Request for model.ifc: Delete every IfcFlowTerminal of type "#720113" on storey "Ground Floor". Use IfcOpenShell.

First a look at what the model holds.

```python
import ifcopenshell
import ifcopenshell.util.element

model = ifcopenshell.open("model.ifc")
print(model.schema)
storey = next(s for s in model.by_type("IfcBuildingStorey") if s.Name == "Ground Floor")
terminals = [e for e in ifcopenshell.util.element.get_decomposition(storey) if e.is_a("IfcFlowTerminal")]
seen = {}
for e in terminals:
    element_type = ifcopenshell.util.element.get_type(e)
    name = element_type.Name if element_type not in (None, e) else None
    seen[name] = seen.get(name, 0) + 1
for name, count in sorted(seen.items(), key=str):
    print(count, "x", name)
```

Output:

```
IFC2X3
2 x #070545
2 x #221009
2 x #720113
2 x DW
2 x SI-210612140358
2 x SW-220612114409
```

```python
import ifcopenshell
import ifcopenshell.api.root
import ifcopenshell.util.element

model = ifcopenshell.open("model.ifc")

storey = next(s for s in model.by_type("IfcBuildingStorey") if s.Name == "Ground Floor")
terminals = [e for e in ifcopenshell.util.element.get_decomposition(storey) if e.is_a("IfcFlowTerminal")]
targets = [e for e in terminals if (t := ifcopenshell.util.element.get_type(e)) not in (None, e) and t.Name == "#720113"]

for e in targets:
    ifcopenshell.api.root.remove_product(model, product=e)
print(len(targets), "removed")

model.write("model_rev.ifc")
```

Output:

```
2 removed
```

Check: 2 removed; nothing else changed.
